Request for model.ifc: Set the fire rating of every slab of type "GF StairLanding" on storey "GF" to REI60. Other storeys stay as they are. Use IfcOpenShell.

First a look at what the model holds.

```python
import ifcopenshell
import ifcopenshell.util.element

model = ifcopenshell.open("model.ifc")
print(model.schema)
storey = next(s for s in model.by_type("IfcBuildingStorey") if s.Name == "GF")
slabs = [e for e in ifcopenshell.util.element.get_decomposition(storey) if e.is_a("IfcSlab")]
seen = {}
for e in slabs:
    element_type = ifcopenshell.util.element.get_type(e)
    key = (element_type.Name if element_type != e and element_type else None, ifcopenshell.util.element.get_pset(e, "Pset_SlabCommon", "FireRating"))
    seen[key] = seen.get(key, 0) + 1
for (name, value), count in sorted(seen.items(), key=str):
    print(count, "x", name, "|", value)
```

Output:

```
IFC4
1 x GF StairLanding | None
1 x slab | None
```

```python
import ifcopenshell
import ifcopenshell.api.pset
import ifcopenshell.util.element

model = ifcopenshell.open("model.ifc")

storey = next(s for s in model.by_type("IfcBuildingStorey") if s.Name == "GF")
slabs = [e for e in ifcopenshell.util.element.get_decomposition(storey) if e.is_a("IfcSlab")]

count = 0
for e in slabs:
    element_type = ifcopenshell.util.element.get_type(e)
    if element_type in (None, e) or element_type.Name != "GF StairLanding":
        continue
    # add_pset returns the element's existing set when there is one.
    pset = ifcopenshell.api.pset.add_pset(model, product=e, name="Pset_SlabCommon")
    ifcopenshell.api.pset.edit_pset(model, pset=pset, properties={"FireRating": "REI60"})
    count += 1

print(count, "slabs updated")

model.write("model_v2.ifc")
```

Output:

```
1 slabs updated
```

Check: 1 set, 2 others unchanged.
